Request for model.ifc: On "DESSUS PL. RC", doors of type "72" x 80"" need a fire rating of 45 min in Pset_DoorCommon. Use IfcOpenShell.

First a look at what the model holds.

```python
import ifcopenshell
import ifcopenshell.util.element

model = ifcopenshell.open("model.ifc")
print(model.schema)
storey = next(s for s in model.by_type("IfcBuildingStorey") if s.Name == "DESSUS PL. RC")
doors = [e for e in ifcopenshell.util.element.get_decomposition(storey) if e.is_a("IfcDoor")]
seen = {}
for e in doors:
    element_type = ifcopenshell.util.element.get_type(e)
    key = (element_type.Name if element_type != e and element_type else None, ifcopenshell.util.element.get_pset(e, "Pset_DoorCommon", "FireRating"))
    seen[key] = seen.get(key, 0) + 1
for (name, value), count in sorted(seen.items(), key=str):
    print(count, "x", name, "|", value)
```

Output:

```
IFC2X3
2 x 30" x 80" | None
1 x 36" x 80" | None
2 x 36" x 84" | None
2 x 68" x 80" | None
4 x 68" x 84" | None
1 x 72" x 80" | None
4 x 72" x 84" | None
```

```python
import ifcopenshell
import ifcopenshell.api.pset
import ifcopenshell.util.element

model = ifcopenshell.open("model.ifc")

storey = next(s for s in model.by_type("IfcBuildingStorey") if s.Name == "DESSUS PL. RC")
doors = [e for e in ifcopenshell.util.element.get_decomposition(storey) if e.is_a("IfcDoor")]

count = 0
for e in doors:
    element_type = ifcopenshell.util.element.get_type(e)
    if element_type in (None, e) or element_type.Name != '72" x 80"':
        continue
    # add_pset returns the element's existing set when there is one.
    pset = ifcopenshell.api.pset.add_pset(model, product=e, name="Pset_DoorCommon")
    ifcopenshell.api.pset.edit_pset(model, pset=pset, properties={"FireRating": "45 min"})
    count += 1

print(count, "doors updated")

model.write("model_rev.ifc")
```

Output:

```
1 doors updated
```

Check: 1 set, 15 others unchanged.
